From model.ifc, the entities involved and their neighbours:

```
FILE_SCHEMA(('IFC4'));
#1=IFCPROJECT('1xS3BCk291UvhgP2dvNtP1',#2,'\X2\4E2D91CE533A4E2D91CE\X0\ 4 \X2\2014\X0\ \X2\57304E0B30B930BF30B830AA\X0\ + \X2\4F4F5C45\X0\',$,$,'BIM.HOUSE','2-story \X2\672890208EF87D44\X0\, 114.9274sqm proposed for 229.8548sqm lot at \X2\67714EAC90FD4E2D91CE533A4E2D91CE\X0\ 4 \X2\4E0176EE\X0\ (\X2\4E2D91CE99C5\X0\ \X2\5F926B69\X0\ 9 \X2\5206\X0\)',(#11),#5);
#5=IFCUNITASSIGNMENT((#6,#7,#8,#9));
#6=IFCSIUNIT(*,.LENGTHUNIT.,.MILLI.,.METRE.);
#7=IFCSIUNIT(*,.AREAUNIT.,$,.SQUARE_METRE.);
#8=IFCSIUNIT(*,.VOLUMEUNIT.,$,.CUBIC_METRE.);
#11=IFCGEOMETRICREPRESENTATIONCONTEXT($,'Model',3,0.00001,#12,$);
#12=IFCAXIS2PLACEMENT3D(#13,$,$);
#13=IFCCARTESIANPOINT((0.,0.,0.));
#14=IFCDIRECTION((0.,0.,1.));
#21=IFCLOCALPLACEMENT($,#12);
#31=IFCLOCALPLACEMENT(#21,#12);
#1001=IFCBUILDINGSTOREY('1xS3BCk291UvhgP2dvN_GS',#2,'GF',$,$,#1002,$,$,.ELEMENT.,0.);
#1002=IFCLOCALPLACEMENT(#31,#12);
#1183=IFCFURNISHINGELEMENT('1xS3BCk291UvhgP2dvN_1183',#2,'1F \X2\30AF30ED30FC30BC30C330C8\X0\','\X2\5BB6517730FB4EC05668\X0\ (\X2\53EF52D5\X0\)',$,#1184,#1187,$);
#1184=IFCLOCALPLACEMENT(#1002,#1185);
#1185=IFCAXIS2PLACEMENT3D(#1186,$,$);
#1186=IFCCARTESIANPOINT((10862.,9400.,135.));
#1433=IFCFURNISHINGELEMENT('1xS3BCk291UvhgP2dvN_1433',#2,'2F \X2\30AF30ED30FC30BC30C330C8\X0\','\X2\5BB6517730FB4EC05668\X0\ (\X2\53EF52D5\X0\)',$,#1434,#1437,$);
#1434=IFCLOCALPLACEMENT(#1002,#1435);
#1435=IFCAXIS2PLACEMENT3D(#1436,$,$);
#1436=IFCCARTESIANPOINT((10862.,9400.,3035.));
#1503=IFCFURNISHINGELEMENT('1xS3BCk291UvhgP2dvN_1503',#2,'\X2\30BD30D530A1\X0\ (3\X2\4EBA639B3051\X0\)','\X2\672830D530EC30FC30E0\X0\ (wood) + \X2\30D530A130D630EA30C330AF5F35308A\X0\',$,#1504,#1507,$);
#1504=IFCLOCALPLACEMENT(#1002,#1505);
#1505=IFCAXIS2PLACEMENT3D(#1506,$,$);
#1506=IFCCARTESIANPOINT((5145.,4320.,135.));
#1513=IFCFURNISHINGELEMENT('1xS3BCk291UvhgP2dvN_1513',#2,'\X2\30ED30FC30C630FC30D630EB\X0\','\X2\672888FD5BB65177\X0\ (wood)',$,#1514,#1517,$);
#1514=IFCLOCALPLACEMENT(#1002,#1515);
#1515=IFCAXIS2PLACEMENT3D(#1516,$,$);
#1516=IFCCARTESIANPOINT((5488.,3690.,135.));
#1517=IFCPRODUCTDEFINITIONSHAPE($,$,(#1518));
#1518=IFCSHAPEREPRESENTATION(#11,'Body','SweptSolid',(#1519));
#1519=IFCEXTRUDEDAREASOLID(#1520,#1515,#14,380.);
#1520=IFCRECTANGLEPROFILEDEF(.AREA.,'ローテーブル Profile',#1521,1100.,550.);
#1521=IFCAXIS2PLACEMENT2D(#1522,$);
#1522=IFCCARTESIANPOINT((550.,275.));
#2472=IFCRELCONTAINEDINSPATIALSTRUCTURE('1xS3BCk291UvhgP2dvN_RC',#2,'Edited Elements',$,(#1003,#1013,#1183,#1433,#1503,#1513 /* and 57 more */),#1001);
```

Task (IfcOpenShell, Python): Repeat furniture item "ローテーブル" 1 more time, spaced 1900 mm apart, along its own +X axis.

```python
import ifcopenshell
import ifcopenshell.api.geometry
import ifcopenshell.api.root
import ifcopenshell.util.element
import ifcopenshell.util.placement

model = ifcopenshell.open("model.ifc")


def reuse_history(source, copy):
    """copy_class also copies each property set's owner history, people and application; keep the originals."""
    for rel in copy.IsDefinedBy:
        if rel.is_a("IfcRelDefinesByProperties") and (history := rel.RelatingPropertyDefinition.OwnerHistory):
            rel.RelatingPropertyDefinition.OwnerHistory = source.OwnerHistory
            ifcopenshell.util.element.remove_deep2(model, history)


source = model.by_id(1513)
base = ifcopenshell.util.placement.get_local_placement(source.ObjectPlacement)
step = base[:3, 0] * 1900.0

for i in range(1, 2):
    copy = ifcopenshell.api.root.copy_class(model, product=source)
    copy.Representation = ifcopenshell.util.element.copy_deep(
        model, source.Representation, exclude=["IfcGeometricRepresentationContext", "IfcRepresentationMap"]
    )
    reuse_history(source, copy)
    matrix = base.copy()
    matrix[:3, 3] += i * step
    print("added at", matrix[:3, 3].round(3) + 0.0)
    ifcopenshell.api.geometry.edit_object_placement(model, product=copy, matrix=matrix, is_si=False)

model.write("model-out.ifc")
```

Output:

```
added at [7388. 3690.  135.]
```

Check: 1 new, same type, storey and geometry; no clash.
